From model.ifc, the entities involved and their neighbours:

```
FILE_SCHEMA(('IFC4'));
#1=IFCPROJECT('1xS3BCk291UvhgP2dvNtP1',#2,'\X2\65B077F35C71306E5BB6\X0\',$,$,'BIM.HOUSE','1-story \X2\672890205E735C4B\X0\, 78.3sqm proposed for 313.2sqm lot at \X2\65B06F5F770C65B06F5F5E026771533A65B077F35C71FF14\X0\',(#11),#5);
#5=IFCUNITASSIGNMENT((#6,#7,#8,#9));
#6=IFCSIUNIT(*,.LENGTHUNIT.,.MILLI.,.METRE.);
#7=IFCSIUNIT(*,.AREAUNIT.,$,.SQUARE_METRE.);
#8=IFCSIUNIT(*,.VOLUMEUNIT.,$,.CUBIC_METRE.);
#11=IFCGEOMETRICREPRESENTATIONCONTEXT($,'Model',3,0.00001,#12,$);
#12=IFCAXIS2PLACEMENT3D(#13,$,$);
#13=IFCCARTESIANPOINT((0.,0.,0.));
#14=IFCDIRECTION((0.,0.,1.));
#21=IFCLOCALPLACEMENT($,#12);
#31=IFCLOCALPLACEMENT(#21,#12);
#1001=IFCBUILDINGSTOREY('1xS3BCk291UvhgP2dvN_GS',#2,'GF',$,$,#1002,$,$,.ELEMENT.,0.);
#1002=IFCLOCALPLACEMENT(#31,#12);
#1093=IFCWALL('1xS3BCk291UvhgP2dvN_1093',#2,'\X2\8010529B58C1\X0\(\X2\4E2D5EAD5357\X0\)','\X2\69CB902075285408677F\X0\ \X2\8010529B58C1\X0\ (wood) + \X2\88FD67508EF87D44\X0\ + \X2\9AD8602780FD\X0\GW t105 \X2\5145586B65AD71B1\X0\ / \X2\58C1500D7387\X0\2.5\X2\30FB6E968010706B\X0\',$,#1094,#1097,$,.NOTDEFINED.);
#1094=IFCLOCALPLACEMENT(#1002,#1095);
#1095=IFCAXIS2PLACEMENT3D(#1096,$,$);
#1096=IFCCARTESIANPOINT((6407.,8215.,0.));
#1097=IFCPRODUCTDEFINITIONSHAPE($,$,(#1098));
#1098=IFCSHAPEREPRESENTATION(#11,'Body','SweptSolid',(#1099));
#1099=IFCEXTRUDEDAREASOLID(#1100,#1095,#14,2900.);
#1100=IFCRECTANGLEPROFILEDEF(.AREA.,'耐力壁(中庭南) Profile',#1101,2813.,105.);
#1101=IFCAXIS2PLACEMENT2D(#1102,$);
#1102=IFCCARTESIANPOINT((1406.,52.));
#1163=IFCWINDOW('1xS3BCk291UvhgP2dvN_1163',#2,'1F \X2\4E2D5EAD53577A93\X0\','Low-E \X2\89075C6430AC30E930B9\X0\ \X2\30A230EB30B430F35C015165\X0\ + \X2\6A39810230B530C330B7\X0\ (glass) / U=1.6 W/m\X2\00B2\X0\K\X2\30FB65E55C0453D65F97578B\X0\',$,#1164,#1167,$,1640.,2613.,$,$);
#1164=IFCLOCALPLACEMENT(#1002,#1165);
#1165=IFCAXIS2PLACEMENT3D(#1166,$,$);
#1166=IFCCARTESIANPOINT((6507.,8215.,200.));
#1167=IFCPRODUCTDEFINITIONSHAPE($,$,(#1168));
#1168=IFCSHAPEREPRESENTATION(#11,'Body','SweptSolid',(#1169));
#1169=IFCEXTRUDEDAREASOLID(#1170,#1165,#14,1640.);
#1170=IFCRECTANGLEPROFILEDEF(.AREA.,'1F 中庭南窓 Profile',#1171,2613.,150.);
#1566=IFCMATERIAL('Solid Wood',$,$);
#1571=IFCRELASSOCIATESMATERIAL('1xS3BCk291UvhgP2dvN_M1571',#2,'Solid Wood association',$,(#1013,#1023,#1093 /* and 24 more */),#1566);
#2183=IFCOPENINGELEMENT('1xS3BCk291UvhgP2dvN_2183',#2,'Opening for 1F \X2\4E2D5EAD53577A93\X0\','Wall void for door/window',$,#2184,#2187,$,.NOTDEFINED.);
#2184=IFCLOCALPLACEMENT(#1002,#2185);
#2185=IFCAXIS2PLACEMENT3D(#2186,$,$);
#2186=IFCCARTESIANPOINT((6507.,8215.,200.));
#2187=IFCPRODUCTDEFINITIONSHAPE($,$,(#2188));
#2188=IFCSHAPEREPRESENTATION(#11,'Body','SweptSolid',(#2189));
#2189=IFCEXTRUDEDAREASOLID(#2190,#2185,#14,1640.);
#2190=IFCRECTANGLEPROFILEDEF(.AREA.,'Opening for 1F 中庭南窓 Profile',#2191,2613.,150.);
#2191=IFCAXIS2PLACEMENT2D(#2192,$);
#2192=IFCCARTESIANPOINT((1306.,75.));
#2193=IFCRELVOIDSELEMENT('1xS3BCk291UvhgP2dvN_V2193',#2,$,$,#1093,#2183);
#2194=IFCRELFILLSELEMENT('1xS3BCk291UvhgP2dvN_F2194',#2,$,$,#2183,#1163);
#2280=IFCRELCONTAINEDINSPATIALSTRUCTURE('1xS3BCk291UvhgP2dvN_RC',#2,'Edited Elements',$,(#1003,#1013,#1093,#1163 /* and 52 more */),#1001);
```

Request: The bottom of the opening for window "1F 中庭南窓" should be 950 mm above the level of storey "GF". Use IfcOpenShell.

```python
import numpy as np
import ifcopenshell
import ifcopenshell.api.geometry
import ifcopenshell.geom
import ifcopenshell.util.element
import ifcopenshell.util.placement
import ifcopenshell.util.shape
import ifcopenshell.util.unit

model = ifcopenshell.open("model.ifc")
unit_scale = ifcopenshell.util.unit.calculate_unit_scale(model)

window = model.by_guid("1xS3BCk291UvhgP2dvN_1163")
opening = window.FillsVoids[0].RelatingOpeningElement
storey = ifcopenshell.util.element.get_container(window, ifc_class="IfcBuildingStorey")
level = ifcopenshell.util.placement.get_local_placement(storey.ObjectPlacement)[2, 3]

# The opening's origin need not be at the sill, so measure its lowest point.
shape = ifcopenshell.geom.create_shape(ifcopenshell.geom.settings(), opening)
bottom = ifcopenshell.util.shape.get_shape_bottom_elevation(shape, shape.geometry) / unit_scale
dz = level + 0.95 / unit_scale - bottom

shift = np.array([0.0, 0.0, dz])
# The window is not placed relative to its opening, so move both.
for product in (opening, window):
    matrix = ifcopenshell.util.placement.get_local_placement(product.ObjectPlacement)
    matrix[:3, 3] += shift
    ifcopenshell.api.geometry.edit_object_placement(model, product=product, matrix=matrix, is_si=False)

print(f"moved by {dz * unit_scale:+.3f} m")

model.write("model_rev.ifc")
```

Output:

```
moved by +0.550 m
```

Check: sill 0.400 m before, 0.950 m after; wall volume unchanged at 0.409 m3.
